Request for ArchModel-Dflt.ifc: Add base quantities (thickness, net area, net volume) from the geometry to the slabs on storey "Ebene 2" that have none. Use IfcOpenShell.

First a look at what the model holds.

```python
import ifcopenshell
import ifcopenshell.util.element
import ifcopenshell.util.unit

model = ifcopenshell.open("ArchModel-Dflt.ifc")
print(model.schema)
for unit_type in ("LENGTHUNIT", "AREAUNIT", "VOLUMEUNIT"):
    print(unit_type, ifcopenshell.util.unit.calculate_unit_scale(model, unit_type))
storey = next(s for s in model.by_type("IfcBuildingStorey") if s.Name == "Ebene 2")
slabs = [e for e in ifcopenshell.util.element.get_decomposition(storey) if e.is_a("IfcSlab")]
for e in sorted(slabs, key=lambda e: e.id()):
    print(e.id(), e.is_a(), e.Name, list(ifcopenshell.util.element.get_psets(e, qtos_only=True)), sep=" | ")
```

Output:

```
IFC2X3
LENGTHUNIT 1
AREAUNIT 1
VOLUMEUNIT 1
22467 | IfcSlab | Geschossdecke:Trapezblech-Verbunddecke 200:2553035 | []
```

```python
import ifcopenshell
import ifcopenshell.api.pset
import ifcopenshell.geom
import ifcopenshell.util.element
import ifcopenshell.util.shape
import ifcopenshell.util.unit

model = ifcopenshell.open("ArchModel-Dflt.ifc")
unit_scale = ifcopenshell.util.unit.calculate_unit_scale(model)
area_scale = ifcopenshell.util.unit.calculate_unit_scale(model, "AREAUNIT")
volume_scale = ifcopenshell.util.unit.calculate_unit_scale(model, "VOLUMEUNIT")
settings = ifcopenshell.geom.settings()

storey = next(s for s in model.by_type("IfcBuildingStorey") if s.Name == "Ebene 2")
slabs = [e for e in ifcopenshell.util.element.get_decomposition(storey) if e.is_a("IfcSlab")]

for e in sorted(slabs, key=lambda e: e.id()):
    if ifcopenshell.util.element.get_psets(e, qtos_only=True, should_inherit=False):
        continue
    # Geometry comes back in metres, in the element's own axes.
    shape = ifcopenshell.geom.create_shape(settings, e)
    values = {
        "Width": ifcopenshell.util.shape.get_z(shape.geometry) / unit_scale,
        "NetArea": ifcopenshell.util.shape.get_footprint_area(shape.geometry) / area_scale,
        "NetVolume": ifcopenshell.util.shape.get_volume(shape.geometry) / volume_scale,
    }
    qto = ifcopenshell.api.pset.add_qto(model, product=e, name="BaseQuantities")
    ifcopenshell.api.pset.edit_qto(model, qto=qto, properties=values)
    print(e.id(), {k: round(v, 3) for k, v in values.items()})

model.write("ArchModel-Dflt_edited.ifc")
```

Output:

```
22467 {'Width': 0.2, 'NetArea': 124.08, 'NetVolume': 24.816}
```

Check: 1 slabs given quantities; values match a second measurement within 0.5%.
